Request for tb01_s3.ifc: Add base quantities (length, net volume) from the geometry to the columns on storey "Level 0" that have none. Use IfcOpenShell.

First a look at what the model holds.

```python
import ifcopenshell
import ifcopenshell.util.element
import ifcopenshell.util.unit

model = ifcopenshell.open("tb01_s3.ifc")
print(model.schema)
for unit_type in ("LENGTHUNIT", "AREAUNIT", "VOLUMEUNIT"):
    print(unit_type, ifcopenshell.util.unit.calculate_unit_scale(model, unit_type))
storey = next(s for s in model.by_type("IfcBuildingStorey") if s.Name == "Level 0")
columns = [e for e in ifcopenshell.util.element.get_decomposition(storey) if e.is_a("IfcColumn")]
for e in sorted(columns, key=lambda e: e.id()):
    print(e.id(), e.is_a(), e.Name, list(ifcopenshell.util.element.get_psets(e, qtos_only=True)), sep=" | ")
```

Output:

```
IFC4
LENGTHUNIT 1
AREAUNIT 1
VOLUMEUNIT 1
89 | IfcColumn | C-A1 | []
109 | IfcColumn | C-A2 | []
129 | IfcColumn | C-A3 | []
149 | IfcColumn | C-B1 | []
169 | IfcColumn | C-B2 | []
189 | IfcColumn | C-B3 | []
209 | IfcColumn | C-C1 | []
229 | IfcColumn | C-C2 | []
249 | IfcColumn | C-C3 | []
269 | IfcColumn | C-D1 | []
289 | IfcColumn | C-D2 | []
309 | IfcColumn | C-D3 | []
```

```python
import ifcopenshell
import ifcopenshell.api.pset
import ifcopenshell.geom
import ifcopenshell.util.element
import ifcopenshell.util.shape
import ifcopenshell.util.unit

model = ifcopenshell.open("tb01_s3.ifc")
unit_scale = ifcopenshell.util.unit.calculate_unit_scale(model)
volume_scale = ifcopenshell.util.unit.calculate_unit_scale(model, "VOLUMEUNIT")
settings = ifcopenshell.geom.settings()

storey = next(s for s in model.by_type("IfcBuildingStorey") if s.Name == "Level 0")
columns = [e for e in ifcopenshell.util.element.get_decomposition(storey) if e.is_a("IfcColumn")]

for e in sorted(columns, key=lambda e: e.id()):
    if ifcopenshell.util.element.get_psets(e, qtos_only=True, should_inherit=False):
        continue
    # Geometry comes back in metres, in the element's own axes.
    shape = ifcopenshell.geom.create_shape(settings, e)
    values = {
        "Length": ifcopenshell.util.shape.get_z(shape.geometry) / unit_scale,
        "NetVolume": ifcopenshell.util.shape.get_volume(shape.geometry) / volume_scale,
    }
    qto = ifcopenshell.api.pset.add_qto(model, product=e, name="Qto_ColumnBaseQuantities")
    ifcopenshell.api.pset.edit_qto(model, qto=qto, properties=values)
    print(e.id(), {k: round(v, 3) for k, v in values.items()})

model.write("tb01_s3_v2.ifc")
```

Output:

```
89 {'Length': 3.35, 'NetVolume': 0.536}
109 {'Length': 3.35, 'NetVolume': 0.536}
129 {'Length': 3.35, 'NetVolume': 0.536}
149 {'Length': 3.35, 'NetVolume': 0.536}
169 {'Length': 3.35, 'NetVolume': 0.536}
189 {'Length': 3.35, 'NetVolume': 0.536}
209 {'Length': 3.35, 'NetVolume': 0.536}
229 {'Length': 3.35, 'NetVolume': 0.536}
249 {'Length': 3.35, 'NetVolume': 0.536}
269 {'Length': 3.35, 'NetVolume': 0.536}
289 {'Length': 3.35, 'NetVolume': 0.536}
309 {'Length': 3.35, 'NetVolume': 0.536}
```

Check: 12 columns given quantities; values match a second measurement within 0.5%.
